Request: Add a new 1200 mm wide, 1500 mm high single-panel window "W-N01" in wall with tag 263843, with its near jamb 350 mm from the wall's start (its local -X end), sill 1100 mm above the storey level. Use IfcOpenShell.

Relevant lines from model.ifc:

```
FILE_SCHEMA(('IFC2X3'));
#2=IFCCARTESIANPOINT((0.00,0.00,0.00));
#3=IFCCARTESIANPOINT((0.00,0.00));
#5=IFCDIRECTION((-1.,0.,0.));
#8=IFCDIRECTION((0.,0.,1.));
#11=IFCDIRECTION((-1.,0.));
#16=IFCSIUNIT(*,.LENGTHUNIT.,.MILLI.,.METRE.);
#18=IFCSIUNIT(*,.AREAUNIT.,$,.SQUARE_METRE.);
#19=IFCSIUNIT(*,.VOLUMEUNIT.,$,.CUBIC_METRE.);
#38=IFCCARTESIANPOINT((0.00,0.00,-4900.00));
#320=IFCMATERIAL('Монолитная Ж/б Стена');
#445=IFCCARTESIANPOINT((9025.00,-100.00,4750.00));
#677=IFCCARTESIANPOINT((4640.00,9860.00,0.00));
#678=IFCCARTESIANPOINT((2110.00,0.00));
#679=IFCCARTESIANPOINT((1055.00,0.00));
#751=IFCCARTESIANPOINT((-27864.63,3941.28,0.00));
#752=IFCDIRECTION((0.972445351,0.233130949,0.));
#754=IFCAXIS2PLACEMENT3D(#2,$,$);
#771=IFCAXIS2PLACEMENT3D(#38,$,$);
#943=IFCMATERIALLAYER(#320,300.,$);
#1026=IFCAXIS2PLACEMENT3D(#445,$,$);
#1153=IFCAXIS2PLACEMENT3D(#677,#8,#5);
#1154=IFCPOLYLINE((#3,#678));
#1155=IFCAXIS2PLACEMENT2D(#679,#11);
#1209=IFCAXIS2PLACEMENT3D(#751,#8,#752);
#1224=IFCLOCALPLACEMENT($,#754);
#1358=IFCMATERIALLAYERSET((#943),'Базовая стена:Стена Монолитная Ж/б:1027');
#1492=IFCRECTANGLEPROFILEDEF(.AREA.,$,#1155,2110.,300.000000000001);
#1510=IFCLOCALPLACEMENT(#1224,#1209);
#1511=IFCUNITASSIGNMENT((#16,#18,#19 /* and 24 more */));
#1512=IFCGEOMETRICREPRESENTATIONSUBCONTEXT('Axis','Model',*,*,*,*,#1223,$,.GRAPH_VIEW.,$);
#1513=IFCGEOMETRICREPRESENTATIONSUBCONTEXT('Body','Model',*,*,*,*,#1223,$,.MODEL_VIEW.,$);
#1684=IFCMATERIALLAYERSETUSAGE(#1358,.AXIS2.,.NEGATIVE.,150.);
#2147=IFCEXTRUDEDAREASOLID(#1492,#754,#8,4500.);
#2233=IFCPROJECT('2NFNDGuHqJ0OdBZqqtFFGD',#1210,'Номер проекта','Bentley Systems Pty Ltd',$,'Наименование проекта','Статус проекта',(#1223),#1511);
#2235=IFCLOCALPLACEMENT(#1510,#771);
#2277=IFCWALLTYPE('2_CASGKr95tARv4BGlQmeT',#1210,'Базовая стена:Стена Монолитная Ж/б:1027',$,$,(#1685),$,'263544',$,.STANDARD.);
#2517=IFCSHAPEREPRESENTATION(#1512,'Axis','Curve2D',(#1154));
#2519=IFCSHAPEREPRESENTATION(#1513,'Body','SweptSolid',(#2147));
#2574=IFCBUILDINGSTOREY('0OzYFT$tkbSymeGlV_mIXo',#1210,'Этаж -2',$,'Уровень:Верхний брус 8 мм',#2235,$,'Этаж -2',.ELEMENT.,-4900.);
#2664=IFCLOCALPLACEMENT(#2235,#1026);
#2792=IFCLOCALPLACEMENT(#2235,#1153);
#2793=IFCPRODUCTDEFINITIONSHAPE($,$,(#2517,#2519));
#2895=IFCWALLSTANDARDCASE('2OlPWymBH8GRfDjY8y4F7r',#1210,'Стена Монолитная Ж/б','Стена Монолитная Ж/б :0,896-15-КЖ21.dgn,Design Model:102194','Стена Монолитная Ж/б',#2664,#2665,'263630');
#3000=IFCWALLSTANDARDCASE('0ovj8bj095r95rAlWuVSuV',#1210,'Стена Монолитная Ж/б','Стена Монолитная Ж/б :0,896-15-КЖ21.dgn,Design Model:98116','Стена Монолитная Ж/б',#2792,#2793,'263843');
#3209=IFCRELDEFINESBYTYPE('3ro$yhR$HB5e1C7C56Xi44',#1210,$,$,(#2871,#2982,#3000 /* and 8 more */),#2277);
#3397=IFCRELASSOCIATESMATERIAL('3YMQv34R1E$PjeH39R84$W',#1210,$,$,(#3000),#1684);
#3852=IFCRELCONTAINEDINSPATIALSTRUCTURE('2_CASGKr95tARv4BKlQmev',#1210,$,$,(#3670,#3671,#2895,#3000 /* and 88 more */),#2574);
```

```python
import numpy as np
import ifcopenshell
import ifcopenshell.api.feature
import ifcopenshell.api.geometry
import ifcopenshell.api.root
import ifcopenshell.api.spatial
import ifcopenshell.api.type
import ifcopenshell.geom
import ifcopenshell.util.element
import ifcopenshell.util.placement
import ifcopenshell.util.representation
import ifcopenshell.util.shape
import ifcopenshell.util.unit

model = ifcopenshell.open("model.ifc")
unit_scale = ifcopenshell.util.unit.calculate_unit_scale(model)
settings = ifcopenshell.geom.settings()


def volume(element):
    """Net volume in cubic metres, openings subtracted."""
    shape = ifcopenshell.geom.create_shape(settings, element)
    return ifcopenshell.util.shape.get_volume(shape.geometry)


wall = model.by_guid("0ovj8bj095r95rAlWuVSuV")
storey = ifcopenshell.util.element.get_container(wall, ifc_class="IfcBuildingStorey")
context = ifcopenshell.util.representation.get_context(model, "Model", "Body", "MODEL_VIEW")
before = volume(wall)

width, height, from_end, sill = 1.2, 1.5, 0.35, 1.1  # metres

# The wall runs along its own X axis, and the end named is its -X end.
wall_shape = ifcopenshell.geom.create_shape(settings, wall)
x, y, z = ifcopenshell.util.shape.get_vertices(wall_shape.geometry).T
start = x.min() + from_end
face, thickness = float(y.min()), float(y.max() - y.min())
wall_matrix = ifcopenshell.util.placement.get_local_placement(wall.ObjectPlacement)
level = ifcopenshell.util.placement.get_local_placement(storey.ObjectPlacement)[2, 3]


def in_wall(x, y):
    """Placement at x, y metres in the wall's axes, at sill height."""
    matrix = wall_matrix.copy()
    matrix[:, 3] = wall_matrix @ np.array([x / unit_scale, y / unit_scale, 0.0, 1.0])
    matrix[2, 3] = level + sill / unit_scale
    return matrix


# Opening: a box that overshoots both wall faces by 50 mm.
opening = ifcopenshell.api.root.create_entity(model, ifc_class="IfcOpeningElement")
box = ifcopenshell.api.geometry.add_wall_representation(
    model, context=context, length=width, height=height, thickness=thickness + 0.1
)
ifcopenshell.api.geometry.assign_representation(model, product=opening, representation=box)
ifcopenshell.api.geometry.edit_object_placement(model, product=opening, matrix=in_wall(start, face - 0.05), is_si=False)
ifcopenshell.api.feature.add_feature(model, feature=opening, element=wall)

window = ifcopenshell.api.root.create_entity(model, ifc_class="IfcWindow", name="W-N01")
window.OverallWidth, window.OverallHeight = width / unit_scale, height / unit_scale
body = ifcopenshell.api.geometry.add_window_representation(
    model,
    context=context,
    overall_width=window.OverallWidth,
    overall_height=window.OverallHeight,
    partition_type="SINGLE_PANEL",
)
ifcopenshell.api.geometry.assign_representation(model, product=window, representation=body)
ifcopenshell.api.spatial.assign_container(model, products=[window], relating_structure=storey)
fills = ifcopenshell.api.feature.add_filling(model, opening=opening, element=window)
fills.OwnerHistory = window.OwnerHistory  # required in IFC2X3

# IFC2X3 keeps the operation on the window style.
style = ifcopenshell.api.root.create_entity(model, ifc_class="IfcWindowStyle", name="W-N01")
style.OperationType, style.ConstructionType = "SINGLE_PANEL", "NOTDEFINED"
style.ParameterTakesPrecedence = style.Sizeable = False
ifcopenshell.api.type.assign_type(model, related_objects=[window], relating_type=style)

# Centre the window in the wall's thickness.
ifcopenshell.api.geometry.edit_object_placement(model, product=window, matrix=in_wall(start, face), is_si=False)
window_shape = ifcopenshell.geom.create_shape(settings, window)
depth = ifcopenshell.util.shape.get_vertices(window_shape.geometry)[:, 1]
offset = face + thickness / 2 - (depth.min() + depth.max()) / 2
ifcopenshell.api.geometry.edit_object_placement(model, product=window, matrix=in_wall(start, offset), is_si=False)

after = volume(wall)

print(f"wall volume {before:.3f} -> {after:.3f} m3")

model.write("model-out.ifc")
```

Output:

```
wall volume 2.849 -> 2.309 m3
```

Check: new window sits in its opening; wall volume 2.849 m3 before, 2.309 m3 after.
